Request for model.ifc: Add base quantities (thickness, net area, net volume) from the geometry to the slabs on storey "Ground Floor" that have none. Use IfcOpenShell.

First a look at what the model holds.

```python
import ifcopenshell
import ifcopenshell.util.element
import ifcopenshell.util.unit

model = ifcopenshell.open("model.ifc")
print(model.schema)
for unit_type in ("LENGTHUNIT", "AREAUNIT", "VOLUMEUNIT"):
    print(unit_type, ifcopenshell.util.unit.calculate_unit_scale(model, unit_type))
storey = next(s for s in model.by_type("IfcBuildingStorey") if s.Name == "Ground Floor")
slabs = [e for e in ifcopenshell.util.element.get_decomposition(storey) if e.is_a("IfcSlab")]
for e in sorted(slabs, key=lambda e: e.id()):
    print(e.id(), e.is_a(), e.Name, list(ifcopenshell.util.element.get_psets(e, qtos_only=True)), sep=" | ")
```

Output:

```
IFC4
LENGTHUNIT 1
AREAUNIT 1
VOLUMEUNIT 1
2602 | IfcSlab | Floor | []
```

```python
import ifcopenshell
import ifcopenshell.api.pset
import ifcopenshell.geom
import ifcopenshell.util.element
import ifcopenshell.util.shape
import ifcopenshell.util.unit

model = ifcopenshell.open("model.ifc")
unit_scale = ifcopenshell.util.unit.calculate_unit_scale(model)
area_scale = ifcopenshell.util.unit.calculate_unit_scale(model, "AREAUNIT")
volume_scale = ifcopenshell.util.unit.calculate_unit_scale(model, "VOLUMEUNIT")
settings = ifcopenshell.geom.settings()

storey = next(s for s in model.by_type("IfcBuildingStorey") if s.Name == "Ground Floor")
slabs = [e for e in ifcopenshell.util.element.get_decomposition(storey) if e.is_a("IfcSlab")]

for e in sorted(slabs, key=lambda e: e.id()):
    if ifcopenshell.util.element.get_psets(e, qtos_only=True, should_inherit=False):
        continue
    # Geometry comes back in metres, in the element's own axes.
    shape = ifcopenshell.geom.create_shape(settings, e)
    values = {
        "Width": ifcopenshell.util.shape.get_z(shape.geometry) / unit_scale,
        "NetArea": ifcopenshell.util.shape.get_footprint_area(shape.geometry) / area_scale,
        "NetVolume": ifcopenshell.util.shape.get_volume(shape.geometry) / volume_scale,
    }
    qto = ifcopenshell.api.pset.add_qto(model, product=e, name="Qto_SlabBaseQuantities")
    ifcopenshell.api.pset.edit_qto(model, qto=qto, properties=values)
    print(e.id(), {k: round(v, 3) for k, v in values.items()})

model.write("model_v2.ifc")
```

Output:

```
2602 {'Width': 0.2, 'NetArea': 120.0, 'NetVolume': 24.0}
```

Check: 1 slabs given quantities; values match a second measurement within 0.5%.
